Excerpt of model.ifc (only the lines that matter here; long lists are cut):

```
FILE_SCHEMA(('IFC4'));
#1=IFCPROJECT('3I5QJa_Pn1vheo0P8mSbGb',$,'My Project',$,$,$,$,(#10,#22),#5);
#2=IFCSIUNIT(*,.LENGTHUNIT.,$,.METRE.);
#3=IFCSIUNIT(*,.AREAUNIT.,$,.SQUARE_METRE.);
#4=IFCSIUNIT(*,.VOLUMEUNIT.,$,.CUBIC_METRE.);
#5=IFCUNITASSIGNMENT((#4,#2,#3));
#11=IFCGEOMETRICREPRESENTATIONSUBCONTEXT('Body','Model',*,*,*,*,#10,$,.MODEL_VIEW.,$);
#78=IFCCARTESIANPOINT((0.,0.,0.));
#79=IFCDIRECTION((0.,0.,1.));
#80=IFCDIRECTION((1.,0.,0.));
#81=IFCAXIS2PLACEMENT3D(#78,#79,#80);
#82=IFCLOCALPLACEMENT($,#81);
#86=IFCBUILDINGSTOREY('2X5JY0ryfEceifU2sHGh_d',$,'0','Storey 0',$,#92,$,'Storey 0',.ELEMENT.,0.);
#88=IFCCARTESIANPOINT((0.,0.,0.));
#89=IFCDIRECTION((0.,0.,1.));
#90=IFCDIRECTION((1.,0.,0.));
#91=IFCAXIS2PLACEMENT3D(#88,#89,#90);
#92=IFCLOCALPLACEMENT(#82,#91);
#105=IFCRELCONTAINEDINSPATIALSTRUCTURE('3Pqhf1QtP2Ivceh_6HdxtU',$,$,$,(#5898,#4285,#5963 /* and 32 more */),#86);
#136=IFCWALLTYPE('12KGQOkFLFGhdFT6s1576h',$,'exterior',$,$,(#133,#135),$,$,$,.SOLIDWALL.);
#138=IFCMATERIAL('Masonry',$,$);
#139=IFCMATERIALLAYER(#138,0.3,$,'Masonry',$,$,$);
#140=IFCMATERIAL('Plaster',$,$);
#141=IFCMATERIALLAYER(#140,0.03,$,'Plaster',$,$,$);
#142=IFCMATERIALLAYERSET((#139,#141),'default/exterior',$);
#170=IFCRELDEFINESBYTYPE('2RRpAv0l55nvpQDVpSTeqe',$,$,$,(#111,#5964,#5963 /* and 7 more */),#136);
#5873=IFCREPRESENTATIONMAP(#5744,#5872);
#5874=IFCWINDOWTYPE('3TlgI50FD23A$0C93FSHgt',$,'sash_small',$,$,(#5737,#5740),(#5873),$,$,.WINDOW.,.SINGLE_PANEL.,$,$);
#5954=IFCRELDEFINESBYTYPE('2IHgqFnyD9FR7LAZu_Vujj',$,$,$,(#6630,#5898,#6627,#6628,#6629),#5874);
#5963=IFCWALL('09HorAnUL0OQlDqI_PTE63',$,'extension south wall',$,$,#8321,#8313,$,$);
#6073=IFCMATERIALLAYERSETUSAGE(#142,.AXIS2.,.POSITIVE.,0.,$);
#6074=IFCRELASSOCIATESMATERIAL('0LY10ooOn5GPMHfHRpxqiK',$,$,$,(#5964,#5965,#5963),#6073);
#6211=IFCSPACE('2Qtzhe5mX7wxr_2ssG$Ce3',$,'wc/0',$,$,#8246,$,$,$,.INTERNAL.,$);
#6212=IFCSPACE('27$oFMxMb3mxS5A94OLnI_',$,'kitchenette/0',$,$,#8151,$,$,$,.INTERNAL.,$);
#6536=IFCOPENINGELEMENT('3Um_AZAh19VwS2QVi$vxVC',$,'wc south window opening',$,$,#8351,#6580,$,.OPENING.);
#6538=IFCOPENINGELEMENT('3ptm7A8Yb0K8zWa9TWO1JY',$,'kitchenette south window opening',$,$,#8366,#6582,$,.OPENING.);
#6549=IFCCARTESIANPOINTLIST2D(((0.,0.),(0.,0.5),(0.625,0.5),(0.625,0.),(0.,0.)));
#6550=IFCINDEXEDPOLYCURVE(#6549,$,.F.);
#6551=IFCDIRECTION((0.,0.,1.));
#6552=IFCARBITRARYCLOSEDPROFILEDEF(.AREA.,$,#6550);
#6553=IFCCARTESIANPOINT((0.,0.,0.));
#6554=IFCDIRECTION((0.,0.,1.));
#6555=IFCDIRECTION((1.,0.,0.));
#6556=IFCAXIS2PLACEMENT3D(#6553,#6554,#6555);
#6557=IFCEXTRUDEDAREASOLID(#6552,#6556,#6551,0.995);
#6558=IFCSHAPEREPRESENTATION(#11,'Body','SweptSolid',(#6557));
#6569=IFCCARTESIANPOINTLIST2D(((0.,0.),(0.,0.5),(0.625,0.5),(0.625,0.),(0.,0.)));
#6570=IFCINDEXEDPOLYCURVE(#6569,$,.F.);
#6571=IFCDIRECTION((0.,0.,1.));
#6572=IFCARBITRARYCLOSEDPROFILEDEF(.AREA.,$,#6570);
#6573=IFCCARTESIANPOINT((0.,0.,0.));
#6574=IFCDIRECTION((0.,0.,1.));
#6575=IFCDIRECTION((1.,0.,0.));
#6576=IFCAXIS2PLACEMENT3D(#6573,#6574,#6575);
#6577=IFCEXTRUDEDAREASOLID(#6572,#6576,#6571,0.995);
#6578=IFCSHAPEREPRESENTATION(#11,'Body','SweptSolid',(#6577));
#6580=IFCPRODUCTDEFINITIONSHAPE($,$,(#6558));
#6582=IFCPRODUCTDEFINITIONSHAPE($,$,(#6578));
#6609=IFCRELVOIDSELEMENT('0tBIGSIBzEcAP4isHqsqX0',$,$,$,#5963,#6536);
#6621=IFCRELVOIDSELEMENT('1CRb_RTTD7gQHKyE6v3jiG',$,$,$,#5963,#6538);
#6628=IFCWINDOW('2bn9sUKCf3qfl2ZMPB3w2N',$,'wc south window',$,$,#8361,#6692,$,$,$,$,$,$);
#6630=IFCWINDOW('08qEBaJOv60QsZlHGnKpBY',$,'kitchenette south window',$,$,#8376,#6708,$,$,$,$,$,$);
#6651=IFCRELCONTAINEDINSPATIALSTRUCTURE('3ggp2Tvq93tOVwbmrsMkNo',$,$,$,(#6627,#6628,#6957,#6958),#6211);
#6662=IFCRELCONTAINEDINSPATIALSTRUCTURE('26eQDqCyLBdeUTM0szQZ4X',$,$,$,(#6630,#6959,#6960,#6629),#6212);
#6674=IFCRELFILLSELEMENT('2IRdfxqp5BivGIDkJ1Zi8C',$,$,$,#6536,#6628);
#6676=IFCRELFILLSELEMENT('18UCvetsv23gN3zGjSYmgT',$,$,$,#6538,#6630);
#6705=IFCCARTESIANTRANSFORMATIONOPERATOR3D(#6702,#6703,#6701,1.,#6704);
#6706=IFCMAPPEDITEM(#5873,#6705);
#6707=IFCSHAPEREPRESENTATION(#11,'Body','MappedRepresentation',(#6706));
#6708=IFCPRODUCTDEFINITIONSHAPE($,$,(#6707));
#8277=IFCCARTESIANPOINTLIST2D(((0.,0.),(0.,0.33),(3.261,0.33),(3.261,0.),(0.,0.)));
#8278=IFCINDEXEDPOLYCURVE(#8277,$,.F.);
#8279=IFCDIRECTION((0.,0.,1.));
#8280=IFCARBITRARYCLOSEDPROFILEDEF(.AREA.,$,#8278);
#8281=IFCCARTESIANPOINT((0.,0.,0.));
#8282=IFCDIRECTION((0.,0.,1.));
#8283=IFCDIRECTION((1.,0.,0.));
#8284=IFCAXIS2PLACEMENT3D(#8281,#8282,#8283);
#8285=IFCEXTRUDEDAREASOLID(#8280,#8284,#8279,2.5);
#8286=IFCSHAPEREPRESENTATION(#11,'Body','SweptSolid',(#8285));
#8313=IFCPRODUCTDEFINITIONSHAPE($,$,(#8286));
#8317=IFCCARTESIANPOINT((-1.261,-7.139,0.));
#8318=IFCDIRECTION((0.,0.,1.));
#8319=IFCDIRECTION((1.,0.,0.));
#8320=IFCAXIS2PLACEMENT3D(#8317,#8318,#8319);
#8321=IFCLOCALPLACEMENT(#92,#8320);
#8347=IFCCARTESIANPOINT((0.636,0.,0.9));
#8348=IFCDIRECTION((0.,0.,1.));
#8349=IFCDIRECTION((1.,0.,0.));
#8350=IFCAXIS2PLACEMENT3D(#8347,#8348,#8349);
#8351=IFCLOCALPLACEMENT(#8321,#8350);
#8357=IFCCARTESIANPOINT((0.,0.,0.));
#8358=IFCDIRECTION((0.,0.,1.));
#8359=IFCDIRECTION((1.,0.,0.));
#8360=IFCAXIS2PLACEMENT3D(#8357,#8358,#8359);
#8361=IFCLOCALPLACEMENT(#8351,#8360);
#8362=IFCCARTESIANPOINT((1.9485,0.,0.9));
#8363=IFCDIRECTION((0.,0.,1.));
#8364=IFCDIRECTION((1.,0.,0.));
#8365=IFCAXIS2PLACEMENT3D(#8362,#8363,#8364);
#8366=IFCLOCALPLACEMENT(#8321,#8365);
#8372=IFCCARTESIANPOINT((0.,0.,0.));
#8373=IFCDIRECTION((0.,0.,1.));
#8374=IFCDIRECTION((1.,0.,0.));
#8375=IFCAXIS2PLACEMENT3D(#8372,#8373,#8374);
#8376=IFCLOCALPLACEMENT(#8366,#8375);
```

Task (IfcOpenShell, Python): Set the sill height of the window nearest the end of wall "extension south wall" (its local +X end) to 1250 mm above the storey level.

```python
import numpy as np
import ifcopenshell
import ifcopenshell.api.geometry
import ifcopenshell.geom
import ifcopenshell.util.element
import ifcopenshell.util.placement
import ifcopenshell.util.shape
import ifcopenshell.util.unit

model = ifcopenshell.open("model.ifc")
unit_scale = ifcopenshell.util.unit.calculate_unit_scale(model)

window = model.by_guid("08qEBaJOv60QsZlHGnKpBY")
opening = window.FillsVoids[0].RelatingOpeningElement
storey = ifcopenshell.util.element.get_container(window, ifc_class="IfcBuildingStorey")
level = ifcopenshell.util.placement.get_local_placement(storey.ObjectPlacement)[2, 3]

# The opening's origin need not be at the sill, so measure its lowest point.
shape = ifcopenshell.geom.create_shape(ifcopenshell.geom.settings(), opening)
bottom = ifcopenshell.util.shape.get_shape_bottom_elevation(shape, shape.geometry) / unit_scale
dz = level + 1.25 / unit_scale - bottom

shift = np.array([0.0, 0.0, dz])
# The window is placed relative to its opening, so it follows when the opening moves.
matrix = ifcopenshell.util.placement.get_local_placement(opening.ObjectPlacement)
matrix[:3, 3] += shift
ifcopenshell.api.geometry.edit_object_placement(
    model, product=opening, matrix=matrix, is_si=False, should_transform_children=True
)

print(f"moved by {dz * unit_scale:+.3f} m")

model.write("model_v2.ifc")
```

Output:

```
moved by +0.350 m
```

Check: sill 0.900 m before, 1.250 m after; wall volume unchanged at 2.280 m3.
